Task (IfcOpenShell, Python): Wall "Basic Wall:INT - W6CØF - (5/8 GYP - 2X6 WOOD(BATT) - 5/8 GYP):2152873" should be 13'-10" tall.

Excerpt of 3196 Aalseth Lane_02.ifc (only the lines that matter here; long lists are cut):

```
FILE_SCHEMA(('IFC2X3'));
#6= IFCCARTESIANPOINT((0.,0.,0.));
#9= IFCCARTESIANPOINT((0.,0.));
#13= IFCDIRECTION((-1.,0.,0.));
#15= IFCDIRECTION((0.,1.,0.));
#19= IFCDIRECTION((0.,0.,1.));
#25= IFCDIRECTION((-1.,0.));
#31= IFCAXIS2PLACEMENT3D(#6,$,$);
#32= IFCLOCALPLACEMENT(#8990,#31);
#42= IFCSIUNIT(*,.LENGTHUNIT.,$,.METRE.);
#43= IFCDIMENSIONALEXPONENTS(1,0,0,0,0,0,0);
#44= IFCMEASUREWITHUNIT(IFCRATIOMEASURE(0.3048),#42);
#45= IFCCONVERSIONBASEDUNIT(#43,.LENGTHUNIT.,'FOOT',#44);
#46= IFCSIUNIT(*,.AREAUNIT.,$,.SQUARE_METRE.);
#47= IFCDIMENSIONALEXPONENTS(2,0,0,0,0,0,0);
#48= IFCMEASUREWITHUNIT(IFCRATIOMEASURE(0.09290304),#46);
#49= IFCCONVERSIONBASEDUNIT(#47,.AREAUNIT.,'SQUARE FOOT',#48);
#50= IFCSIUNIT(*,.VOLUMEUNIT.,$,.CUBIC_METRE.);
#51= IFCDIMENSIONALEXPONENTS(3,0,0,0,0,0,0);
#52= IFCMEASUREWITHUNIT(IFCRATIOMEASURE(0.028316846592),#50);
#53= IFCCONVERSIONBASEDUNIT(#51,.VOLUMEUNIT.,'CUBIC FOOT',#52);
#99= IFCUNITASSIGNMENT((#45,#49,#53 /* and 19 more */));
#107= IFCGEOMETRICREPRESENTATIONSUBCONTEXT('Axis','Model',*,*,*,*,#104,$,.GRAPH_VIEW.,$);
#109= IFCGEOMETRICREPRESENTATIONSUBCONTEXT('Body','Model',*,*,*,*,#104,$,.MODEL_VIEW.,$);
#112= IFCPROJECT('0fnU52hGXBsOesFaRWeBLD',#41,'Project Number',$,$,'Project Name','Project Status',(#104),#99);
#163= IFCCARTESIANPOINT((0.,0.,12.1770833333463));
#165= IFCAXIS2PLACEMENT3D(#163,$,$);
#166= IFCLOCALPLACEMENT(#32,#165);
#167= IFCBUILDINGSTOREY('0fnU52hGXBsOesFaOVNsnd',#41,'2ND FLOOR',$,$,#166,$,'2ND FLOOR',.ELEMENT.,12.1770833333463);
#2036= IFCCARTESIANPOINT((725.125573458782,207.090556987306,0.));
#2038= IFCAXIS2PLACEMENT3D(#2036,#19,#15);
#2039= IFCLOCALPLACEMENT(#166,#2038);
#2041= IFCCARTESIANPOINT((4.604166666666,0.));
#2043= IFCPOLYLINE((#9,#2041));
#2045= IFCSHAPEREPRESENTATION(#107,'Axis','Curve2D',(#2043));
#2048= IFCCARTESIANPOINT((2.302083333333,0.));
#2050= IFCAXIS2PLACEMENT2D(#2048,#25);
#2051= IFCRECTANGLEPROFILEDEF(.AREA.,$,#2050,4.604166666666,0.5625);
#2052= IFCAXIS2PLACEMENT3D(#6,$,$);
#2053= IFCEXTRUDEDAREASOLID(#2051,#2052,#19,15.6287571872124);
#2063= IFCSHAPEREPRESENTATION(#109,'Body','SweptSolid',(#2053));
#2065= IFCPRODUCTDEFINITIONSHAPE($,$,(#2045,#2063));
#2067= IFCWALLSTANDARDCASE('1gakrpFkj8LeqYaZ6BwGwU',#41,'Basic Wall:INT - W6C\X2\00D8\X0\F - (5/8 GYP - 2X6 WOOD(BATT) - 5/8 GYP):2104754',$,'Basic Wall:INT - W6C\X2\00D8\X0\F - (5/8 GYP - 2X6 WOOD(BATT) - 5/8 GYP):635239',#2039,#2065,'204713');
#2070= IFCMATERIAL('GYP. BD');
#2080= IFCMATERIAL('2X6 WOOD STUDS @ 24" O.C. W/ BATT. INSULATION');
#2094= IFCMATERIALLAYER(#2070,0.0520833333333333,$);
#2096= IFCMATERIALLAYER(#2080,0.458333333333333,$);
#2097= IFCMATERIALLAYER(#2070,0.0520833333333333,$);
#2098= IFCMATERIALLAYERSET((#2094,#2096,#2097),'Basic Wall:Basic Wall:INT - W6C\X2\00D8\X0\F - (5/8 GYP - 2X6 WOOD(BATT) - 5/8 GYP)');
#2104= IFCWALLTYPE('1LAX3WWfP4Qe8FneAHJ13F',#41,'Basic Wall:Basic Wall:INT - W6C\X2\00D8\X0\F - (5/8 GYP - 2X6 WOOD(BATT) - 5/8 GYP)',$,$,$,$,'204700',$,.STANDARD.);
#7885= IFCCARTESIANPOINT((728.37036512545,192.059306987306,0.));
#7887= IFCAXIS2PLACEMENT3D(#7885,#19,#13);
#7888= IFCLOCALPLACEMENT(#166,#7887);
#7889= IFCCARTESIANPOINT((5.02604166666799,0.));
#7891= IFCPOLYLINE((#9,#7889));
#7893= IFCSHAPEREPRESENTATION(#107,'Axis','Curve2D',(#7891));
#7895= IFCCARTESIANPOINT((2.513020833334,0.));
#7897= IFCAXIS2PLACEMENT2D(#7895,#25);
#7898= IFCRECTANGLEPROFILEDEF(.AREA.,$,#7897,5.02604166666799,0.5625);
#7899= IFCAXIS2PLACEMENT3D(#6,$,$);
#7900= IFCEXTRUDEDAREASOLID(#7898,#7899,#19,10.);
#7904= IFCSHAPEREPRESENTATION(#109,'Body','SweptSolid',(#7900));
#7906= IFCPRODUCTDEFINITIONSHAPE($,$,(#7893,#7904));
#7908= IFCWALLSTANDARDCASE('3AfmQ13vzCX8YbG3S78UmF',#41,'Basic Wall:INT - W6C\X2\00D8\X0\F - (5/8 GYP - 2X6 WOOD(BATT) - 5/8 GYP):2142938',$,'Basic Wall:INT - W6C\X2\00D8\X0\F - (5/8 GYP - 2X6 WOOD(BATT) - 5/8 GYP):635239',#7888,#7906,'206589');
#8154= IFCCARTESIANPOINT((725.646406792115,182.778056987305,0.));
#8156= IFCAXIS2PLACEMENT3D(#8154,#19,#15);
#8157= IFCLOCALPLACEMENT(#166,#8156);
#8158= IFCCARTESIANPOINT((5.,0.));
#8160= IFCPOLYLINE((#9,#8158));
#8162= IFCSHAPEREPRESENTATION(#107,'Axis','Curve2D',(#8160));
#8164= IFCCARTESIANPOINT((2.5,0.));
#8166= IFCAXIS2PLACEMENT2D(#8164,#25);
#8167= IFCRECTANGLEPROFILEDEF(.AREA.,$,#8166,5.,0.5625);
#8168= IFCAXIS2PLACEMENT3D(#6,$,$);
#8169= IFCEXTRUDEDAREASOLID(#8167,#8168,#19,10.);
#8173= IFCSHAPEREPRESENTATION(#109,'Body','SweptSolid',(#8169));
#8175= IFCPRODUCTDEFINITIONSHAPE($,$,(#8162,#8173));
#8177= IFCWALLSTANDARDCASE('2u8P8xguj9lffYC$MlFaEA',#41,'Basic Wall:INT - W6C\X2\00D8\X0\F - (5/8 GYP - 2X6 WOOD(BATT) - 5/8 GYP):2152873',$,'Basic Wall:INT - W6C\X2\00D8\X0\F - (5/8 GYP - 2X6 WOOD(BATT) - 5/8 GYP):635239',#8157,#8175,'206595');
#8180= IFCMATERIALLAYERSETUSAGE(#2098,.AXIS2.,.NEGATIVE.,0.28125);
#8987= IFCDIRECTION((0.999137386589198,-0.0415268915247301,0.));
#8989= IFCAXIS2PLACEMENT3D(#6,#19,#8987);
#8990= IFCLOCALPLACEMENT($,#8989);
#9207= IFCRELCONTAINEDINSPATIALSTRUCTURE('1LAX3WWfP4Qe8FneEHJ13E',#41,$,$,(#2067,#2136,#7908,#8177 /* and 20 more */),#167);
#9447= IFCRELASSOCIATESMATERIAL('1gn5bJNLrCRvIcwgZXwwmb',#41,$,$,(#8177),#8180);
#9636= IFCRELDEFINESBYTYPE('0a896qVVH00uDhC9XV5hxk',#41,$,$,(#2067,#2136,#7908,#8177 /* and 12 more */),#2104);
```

```python
import ifcopenshell
import ifcopenshell.geom
import ifcopenshell.util.representation
import ifcopenshell.util.shape
import ifcopenshell.util.unit

model = ifcopenshell.open("3196 Aalseth Lane_02.ifc")
unit_scale = ifcopenshell.util.unit.calculate_unit_scale(model)
settings = ifcopenshell.geom.settings()


def volume(element):
    """Net volume in cubic metres, openings subtracted."""
    shape = ifcopenshell.geom.create_shape(settings, element)
    return ifcopenshell.util.shape.get_volume(shape.geometry)


wall = model.by_guid("2u8P8xguj9lffYC$MlFaEA")
before = volume(wall)

body = ifcopenshell.util.representation.get_representation(wall, "Model", "Body")
solid = body.Items[0]
old_height = solid.Depth
solid.Depth = 166 * 0.0254 / unit_scale
after = volume(wall)

print(f"height {old_height:g} -> {solid.Depth:g}, volume {before:.3f} -> {after:.3f} m3")

model.write("3196 Aalseth Lane_02_edited.ifc")
```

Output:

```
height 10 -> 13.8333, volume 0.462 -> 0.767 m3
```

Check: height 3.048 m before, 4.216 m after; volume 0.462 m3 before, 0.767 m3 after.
